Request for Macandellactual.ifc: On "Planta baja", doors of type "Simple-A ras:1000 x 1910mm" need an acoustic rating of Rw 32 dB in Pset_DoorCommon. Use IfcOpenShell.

First a look at what the model holds.

```python
import ifcopenshell
import ifcopenshell.util.element

model = ifcopenshell.open("Macandellactual.ifc")
print(model.schema)
storey = next(s for s in model.by_type("IfcBuildingStorey") if s.Name == "Planta baja")
doors = [e for e in ifcopenshell.util.element.get_decomposition(storey) if e.is_a("IfcDoor")]
seen = {}
for e in doors:
    element_type = ifcopenshell.util.element.get_type(e)
    key = (element_type.Name if element_type != e and element_type else None, ifcopenshell.util.element.get_pset(e, "Pset_DoorCommon", "AcousticRating"))
    seen[key] = seen.get(key, 0) + 1
for (name, value), count in sorted(seen.items(), key=str):
    print(count, "x", name, "|", value)
```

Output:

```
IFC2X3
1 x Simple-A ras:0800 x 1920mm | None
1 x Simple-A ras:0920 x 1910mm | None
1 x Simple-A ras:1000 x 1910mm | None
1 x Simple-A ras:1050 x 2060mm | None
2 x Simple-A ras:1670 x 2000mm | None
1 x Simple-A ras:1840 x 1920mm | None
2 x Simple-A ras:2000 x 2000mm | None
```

```python
import ifcopenshell
import ifcopenshell.api.pset
import ifcopenshell.util.element

model = ifcopenshell.open("Macandellactual.ifc")

storey = next(s for s in model.by_type("IfcBuildingStorey") if s.Name == "Planta baja")
doors = [e for e in ifcopenshell.util.element.get_decomposition(storey) if e.is_a("IfcDoor")]

count = 0
for e in doors:
    element_type = ifcopenshell.util.element.get_type(e)
    if element_type in (None, e) or element_type.Name != "Simple-A ras:1000 x 1910mm":
        continue
    # add_pset returns the element's existing set when there is one.
    pset = ifcopenshell.api.pset.add_pset(model, product=e, name="Pset_DoorCommon")
    ifcopenshell.api.pset.edit_pset(model, pset=pset, properties={"AcousticRating": "Rw 32 dB"})
    count += 1

print(count, "doors updated")

model.write("Macandellactual_rev.ifc")
```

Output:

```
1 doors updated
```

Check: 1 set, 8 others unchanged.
